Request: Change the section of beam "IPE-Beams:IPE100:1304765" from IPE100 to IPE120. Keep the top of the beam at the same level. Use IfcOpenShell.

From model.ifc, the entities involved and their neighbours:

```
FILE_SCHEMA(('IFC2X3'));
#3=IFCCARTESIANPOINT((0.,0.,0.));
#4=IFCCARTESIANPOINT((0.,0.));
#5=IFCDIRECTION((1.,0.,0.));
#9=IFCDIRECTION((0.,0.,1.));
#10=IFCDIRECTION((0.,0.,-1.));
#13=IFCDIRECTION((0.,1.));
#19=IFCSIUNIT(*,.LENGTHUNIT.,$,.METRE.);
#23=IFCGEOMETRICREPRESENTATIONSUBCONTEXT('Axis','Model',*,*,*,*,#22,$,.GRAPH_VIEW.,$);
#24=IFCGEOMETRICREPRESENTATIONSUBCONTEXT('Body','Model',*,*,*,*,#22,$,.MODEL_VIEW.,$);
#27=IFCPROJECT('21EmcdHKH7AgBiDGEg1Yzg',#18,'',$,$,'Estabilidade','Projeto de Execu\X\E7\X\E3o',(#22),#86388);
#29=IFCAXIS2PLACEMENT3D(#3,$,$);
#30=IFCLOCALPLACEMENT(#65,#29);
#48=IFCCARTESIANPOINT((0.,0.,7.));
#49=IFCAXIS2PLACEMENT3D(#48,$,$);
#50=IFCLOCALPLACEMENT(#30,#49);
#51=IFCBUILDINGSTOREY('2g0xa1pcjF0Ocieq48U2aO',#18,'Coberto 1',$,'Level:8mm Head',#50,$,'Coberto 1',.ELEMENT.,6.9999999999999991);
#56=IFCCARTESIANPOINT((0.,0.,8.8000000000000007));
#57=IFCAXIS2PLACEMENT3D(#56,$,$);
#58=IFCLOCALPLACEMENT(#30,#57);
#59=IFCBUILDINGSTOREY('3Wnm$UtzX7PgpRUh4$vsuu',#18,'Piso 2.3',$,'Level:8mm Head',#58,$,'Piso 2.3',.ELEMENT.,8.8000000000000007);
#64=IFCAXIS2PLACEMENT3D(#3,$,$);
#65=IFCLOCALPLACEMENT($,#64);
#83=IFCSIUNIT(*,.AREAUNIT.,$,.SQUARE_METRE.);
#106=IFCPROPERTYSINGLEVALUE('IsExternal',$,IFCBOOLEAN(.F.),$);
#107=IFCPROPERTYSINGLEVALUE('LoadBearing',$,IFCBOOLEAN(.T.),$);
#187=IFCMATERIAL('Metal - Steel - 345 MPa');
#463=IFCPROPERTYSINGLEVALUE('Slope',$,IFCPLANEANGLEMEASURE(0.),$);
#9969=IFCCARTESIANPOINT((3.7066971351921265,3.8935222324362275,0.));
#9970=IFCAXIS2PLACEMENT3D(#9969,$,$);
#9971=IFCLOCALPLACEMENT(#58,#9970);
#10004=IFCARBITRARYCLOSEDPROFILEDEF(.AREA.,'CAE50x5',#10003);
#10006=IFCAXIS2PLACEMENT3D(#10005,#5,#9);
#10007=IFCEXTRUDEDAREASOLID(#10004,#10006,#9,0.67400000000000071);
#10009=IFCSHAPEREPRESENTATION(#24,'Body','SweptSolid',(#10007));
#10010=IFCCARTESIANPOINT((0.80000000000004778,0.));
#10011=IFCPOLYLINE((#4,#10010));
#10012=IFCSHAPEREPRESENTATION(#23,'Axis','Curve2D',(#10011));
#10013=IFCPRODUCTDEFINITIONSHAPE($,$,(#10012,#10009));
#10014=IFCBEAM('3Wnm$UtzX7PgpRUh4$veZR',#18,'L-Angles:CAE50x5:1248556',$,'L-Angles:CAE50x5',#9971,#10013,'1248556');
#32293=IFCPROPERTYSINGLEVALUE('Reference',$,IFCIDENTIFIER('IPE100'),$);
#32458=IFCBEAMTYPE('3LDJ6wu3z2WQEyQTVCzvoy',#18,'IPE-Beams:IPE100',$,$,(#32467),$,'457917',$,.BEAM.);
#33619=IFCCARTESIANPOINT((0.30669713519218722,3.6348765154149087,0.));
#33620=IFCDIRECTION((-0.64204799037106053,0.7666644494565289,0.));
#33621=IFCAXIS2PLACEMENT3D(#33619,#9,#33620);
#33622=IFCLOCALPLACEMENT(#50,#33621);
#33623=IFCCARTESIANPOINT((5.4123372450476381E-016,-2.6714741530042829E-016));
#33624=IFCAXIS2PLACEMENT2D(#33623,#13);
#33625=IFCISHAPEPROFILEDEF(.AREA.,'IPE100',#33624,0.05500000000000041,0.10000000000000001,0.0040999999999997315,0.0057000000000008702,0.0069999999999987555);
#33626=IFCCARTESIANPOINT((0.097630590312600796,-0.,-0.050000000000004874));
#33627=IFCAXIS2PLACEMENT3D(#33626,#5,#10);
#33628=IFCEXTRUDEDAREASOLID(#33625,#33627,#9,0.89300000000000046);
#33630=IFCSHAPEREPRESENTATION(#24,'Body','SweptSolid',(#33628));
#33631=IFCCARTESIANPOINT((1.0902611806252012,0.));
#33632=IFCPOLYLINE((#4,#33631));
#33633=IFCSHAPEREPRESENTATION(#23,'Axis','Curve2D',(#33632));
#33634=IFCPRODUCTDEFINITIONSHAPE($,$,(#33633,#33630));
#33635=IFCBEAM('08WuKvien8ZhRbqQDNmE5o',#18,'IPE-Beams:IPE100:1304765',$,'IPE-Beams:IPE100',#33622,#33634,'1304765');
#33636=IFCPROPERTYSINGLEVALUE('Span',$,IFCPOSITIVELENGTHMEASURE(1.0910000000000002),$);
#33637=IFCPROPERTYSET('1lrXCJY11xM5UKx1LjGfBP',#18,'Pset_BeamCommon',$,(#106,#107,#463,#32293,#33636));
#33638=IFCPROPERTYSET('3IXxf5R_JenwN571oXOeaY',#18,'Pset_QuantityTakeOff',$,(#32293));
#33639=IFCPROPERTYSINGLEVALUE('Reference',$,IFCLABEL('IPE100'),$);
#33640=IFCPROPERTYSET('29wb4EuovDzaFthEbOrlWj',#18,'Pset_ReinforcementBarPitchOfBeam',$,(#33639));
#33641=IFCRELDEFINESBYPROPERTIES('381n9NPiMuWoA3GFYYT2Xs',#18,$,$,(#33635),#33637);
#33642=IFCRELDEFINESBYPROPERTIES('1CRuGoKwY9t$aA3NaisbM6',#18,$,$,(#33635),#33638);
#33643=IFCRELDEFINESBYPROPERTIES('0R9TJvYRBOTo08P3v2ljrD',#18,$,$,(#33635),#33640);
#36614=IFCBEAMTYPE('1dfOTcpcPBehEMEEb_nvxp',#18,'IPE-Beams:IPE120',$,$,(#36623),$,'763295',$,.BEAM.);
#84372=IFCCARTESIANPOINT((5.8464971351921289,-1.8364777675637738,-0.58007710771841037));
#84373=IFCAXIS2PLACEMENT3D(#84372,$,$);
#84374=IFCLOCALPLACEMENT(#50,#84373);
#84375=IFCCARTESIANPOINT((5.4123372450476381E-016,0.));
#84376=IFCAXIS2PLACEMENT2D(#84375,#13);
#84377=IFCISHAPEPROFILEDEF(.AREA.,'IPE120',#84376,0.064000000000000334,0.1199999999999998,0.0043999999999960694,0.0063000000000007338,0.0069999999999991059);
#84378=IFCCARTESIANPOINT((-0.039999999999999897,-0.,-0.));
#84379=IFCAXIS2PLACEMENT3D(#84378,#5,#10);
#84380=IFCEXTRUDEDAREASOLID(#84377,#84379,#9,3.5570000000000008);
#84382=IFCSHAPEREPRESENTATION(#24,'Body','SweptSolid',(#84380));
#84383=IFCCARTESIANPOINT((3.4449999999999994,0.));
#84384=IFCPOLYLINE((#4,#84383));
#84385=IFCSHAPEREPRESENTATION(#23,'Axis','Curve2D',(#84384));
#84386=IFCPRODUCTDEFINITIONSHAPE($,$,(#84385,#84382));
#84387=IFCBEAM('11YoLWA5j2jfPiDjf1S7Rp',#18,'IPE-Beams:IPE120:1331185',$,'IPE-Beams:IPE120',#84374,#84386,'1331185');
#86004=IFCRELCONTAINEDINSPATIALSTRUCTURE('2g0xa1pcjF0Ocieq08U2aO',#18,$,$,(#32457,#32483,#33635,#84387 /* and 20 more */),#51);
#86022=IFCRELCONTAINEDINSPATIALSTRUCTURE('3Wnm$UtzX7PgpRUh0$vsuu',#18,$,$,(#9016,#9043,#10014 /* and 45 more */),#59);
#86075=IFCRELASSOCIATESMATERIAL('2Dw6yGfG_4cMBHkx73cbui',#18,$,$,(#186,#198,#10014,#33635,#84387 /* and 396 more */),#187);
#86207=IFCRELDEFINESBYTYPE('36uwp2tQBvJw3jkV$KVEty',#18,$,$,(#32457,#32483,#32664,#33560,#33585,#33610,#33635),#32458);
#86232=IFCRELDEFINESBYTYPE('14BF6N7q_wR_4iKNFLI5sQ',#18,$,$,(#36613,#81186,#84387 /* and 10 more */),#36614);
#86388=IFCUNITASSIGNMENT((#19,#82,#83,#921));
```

```python
import ifcopenshell
import ifcopenshell.api.pset
import ifcopenshell.api.type
import ifcopenshell.util.element
import ifcopenshell.util.representation

model = ifcopenshell.open("model.ifc")

member = model.by_guid("08WuKvien8ZhRbqQDNmE5o")
source = next(p for p in model.by_type("IfcIShapeProfileDef") if p.ProfileName == "IPE120")

body = ifcopenshell.util.representation.get_representation(member, "Model", "Body")
solid = body.Items[0]
old_profile = solid.SweptArea

# Copy the section's sizes but keep this member's own profile position.
profile = ifcopenshell.util.element.copy(model, source)
# Profiles are centred, so shift by half the change in depth to hold the top.
shift = (old_profile.OverallDepth - profile.OverallDepth) / 2
x, y = old_profile.Position.Location.Coordinates
up = (-1.0, 0.0)  # upwards, in the solid's own plane
location = model.createIfcCartesianPoint((x + up[0] * shift, y + up[1] * shift))
profile.Position = model.createIfcAxis2Placement2D(location, old_profile.Position.RefDirection)
solid.SweptArea = profile
if not model.get_total_inverses(old_profile):
    ifcopenshell.util.element.remove_deep2(model, old_profile)

new_type = model.by_guid("1dfOTcpcPBehEMEEb_nvxp")
ifcopenshell.api.type.assign_type(
    model, related_objects=[member], relating_type=new_type, should_map_representations=False
)
member.Name = member.Name.replace("IPE100", "IPE120")
member.ObjectType = "IPE-Beams:IPE120"
pset = model.by_id(ifcopenshell.util.element.get_pset(member, "Pset_BeamCommon", should_inherit=False)["id"])
ifcopenshell.api.pset.edit_pset(model, pset=pset, properties={"Reference": "IPE120"})
pset = model.by_id(ifcopenshell.util.element.get_pset(member, "Pset_QuantityTakeOff", should_inherit=False)["id"])
ifcopenshell.api.pset.edit_pset(model, pset=pset, properties={"Reference": "IPE120"})
pset = model.by_id(ifcopenshell.util.element.get_pset(member, "Pset_ReinforcementBarPitchOfBeam", should_inherit=False)["id"])
ifcopenshell.api.pset.edit_pset(model, pset=pset, properties={"Reference": "IPE120"})

print(solid.SweptArea)

model.write("model_v2.ifc")
```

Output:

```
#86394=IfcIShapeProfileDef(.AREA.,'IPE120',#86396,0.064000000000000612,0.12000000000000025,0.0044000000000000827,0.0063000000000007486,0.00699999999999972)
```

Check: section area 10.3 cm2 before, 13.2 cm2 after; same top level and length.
